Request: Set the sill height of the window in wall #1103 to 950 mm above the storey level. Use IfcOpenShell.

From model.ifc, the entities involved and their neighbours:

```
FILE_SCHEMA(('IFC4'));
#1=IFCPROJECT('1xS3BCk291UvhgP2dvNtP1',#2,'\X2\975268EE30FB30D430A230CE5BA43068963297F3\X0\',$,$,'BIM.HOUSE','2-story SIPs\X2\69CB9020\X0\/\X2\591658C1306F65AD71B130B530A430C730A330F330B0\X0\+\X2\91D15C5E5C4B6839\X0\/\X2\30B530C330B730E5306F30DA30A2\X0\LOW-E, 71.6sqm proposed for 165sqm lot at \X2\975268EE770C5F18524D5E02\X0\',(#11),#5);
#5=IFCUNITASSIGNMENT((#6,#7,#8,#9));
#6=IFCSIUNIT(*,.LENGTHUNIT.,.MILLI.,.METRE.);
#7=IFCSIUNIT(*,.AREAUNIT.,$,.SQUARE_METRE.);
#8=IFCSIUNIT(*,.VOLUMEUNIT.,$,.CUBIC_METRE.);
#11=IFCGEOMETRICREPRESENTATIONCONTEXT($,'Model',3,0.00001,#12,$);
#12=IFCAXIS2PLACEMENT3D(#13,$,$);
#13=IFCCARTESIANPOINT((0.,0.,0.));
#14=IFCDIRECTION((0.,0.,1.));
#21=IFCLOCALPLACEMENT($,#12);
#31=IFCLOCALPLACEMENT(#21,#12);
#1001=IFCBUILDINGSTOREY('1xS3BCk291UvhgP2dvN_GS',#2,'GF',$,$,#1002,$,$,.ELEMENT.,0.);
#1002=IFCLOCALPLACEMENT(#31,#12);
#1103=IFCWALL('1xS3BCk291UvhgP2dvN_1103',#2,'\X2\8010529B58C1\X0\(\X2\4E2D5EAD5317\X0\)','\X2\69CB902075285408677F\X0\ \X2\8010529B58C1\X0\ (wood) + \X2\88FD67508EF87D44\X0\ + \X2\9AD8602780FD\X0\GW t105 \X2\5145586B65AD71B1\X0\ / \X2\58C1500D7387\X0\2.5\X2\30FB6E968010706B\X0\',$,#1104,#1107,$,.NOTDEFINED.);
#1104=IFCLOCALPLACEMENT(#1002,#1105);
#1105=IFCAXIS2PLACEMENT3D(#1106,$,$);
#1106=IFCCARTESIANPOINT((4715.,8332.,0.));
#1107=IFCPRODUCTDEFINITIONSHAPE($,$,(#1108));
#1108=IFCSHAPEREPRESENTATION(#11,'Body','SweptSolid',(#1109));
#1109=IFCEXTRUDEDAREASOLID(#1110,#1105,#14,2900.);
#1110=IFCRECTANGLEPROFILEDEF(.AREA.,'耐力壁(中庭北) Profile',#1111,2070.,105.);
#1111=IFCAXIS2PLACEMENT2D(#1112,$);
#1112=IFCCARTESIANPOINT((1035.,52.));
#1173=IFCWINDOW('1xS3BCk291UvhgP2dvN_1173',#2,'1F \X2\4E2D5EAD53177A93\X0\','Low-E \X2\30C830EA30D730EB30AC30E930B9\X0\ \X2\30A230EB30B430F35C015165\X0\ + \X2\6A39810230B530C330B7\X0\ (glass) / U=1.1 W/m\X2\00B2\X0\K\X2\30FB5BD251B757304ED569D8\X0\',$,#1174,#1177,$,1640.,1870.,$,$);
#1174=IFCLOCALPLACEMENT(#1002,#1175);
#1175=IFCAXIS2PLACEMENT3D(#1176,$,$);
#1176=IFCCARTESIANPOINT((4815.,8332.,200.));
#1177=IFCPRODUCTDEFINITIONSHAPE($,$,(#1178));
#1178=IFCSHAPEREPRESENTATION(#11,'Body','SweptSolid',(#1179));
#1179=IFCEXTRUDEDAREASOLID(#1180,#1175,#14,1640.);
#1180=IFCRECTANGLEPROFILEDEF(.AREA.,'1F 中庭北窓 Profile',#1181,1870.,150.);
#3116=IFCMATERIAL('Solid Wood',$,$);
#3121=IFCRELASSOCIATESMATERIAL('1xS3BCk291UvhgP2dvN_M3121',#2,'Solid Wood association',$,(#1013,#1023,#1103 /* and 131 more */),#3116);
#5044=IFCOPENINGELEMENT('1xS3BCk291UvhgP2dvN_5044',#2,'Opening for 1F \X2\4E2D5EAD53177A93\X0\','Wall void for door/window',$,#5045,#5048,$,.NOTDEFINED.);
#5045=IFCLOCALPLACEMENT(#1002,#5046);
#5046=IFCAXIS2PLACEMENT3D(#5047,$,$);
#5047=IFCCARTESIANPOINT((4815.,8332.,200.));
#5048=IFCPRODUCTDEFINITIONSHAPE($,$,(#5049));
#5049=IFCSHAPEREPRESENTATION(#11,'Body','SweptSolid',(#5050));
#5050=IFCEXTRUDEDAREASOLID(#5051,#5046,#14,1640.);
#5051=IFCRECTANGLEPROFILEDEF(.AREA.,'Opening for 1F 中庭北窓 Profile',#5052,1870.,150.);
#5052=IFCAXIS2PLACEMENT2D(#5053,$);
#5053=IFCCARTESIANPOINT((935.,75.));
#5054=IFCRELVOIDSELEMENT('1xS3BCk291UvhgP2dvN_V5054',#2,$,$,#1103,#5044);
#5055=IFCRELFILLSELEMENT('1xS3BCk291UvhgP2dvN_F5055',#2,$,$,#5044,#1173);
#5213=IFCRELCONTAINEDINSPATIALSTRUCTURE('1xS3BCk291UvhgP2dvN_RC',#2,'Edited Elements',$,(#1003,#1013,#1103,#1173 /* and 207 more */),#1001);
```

```python
import numpy as np
import ifcopenshell
import ifcopenshell.api.geometry
import ifcopenshell.geom
import ifcopenshell.util.element
import ifcopenshell.util.placement
import ifcopenshell.util.shape
import ifcopenshell.util.unit

model = ifcopenshell.open("model.ifc")
unit_scale = ifcopenshell.util.unit.calculate_unit_scale(model)

window = model.by_guid("1xS3BCk291UvhgP2dvN_1173")
opening = window.FillsVoids[0].RelatingOpeningElement
storey = ifcopenshell.util.element.get_container(window, ifc_class="IfcBuildingStorey")
level = ifcopenshell.util.placement.get_local_placement(storey.ObjectPlacement)[2, 3]

# The opening's origin need not be at the sill, so measure its lowest point.
shape = ifcopenshell.geom.create_shape(ifcopenshell.geom.settings(), opening)
bottom = ifcopenshell.util.shape.get_shape_bottom_elevation(shape, shape.geometry) / unit_scale
dz = level + 950.0 - bottom

shift = np.array([0.0, 0.0, dz])
# The window is not placed relative to its opening, so move both.
for product in (opening, window):
    matrix = ifcopenshell.util.placement.get_local_placement(product.ObjectPlacement)
    matrix[:3, 3] += shift
    ifcopenshell.api.geometry.edit_object_placement(model, product=product, matrix=matrix, is_si=False)

print(f"moved by {dz * unit_scale:+.3f} m")

model.write("model_updated.ifc")
```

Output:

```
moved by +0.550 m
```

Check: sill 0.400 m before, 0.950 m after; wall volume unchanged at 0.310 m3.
